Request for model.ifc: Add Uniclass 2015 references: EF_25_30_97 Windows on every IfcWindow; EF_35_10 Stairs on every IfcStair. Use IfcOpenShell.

First a look at what the model holds.

```python
import ifcopenshell

model = ifcopenshell.open("model.ifc")
print(model.schema)
print("classifications:", [c.Name for c in model.by_type("IfcClassification")])
for ifc_class in ("IfcDoor", "IfcRoof", "IfcStair", "IfcWall", "IfcWindow"):
    print(ifc_class, len(model.by_type(ifc_class)))
```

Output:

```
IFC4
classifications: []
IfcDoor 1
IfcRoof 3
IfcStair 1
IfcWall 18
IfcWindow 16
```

```python
import ifcopenshell
import ifcopenshell.api.classification

model = ifcopenshell.open("model.ifc")

system = ifcopenshell.api.classification.add_classification(model, classification="Uniclass 2015")

codes = {
    "IfcWindow": ("EF_25_30_97", "Windows"),
    "IfcStair": ("EF_35_10", "Stairs"),
}
for ifc_class, (code, name) in codes.items():
    products = model.by_type(ifc_class)
    ifcopenshell.api.classification.add_reference(
        model, products=products, classification=system, identification=code, name=name
    )
    print(code, len(products))

model.write("model_rev.ifc")
```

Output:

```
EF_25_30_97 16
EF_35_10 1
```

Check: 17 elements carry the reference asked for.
